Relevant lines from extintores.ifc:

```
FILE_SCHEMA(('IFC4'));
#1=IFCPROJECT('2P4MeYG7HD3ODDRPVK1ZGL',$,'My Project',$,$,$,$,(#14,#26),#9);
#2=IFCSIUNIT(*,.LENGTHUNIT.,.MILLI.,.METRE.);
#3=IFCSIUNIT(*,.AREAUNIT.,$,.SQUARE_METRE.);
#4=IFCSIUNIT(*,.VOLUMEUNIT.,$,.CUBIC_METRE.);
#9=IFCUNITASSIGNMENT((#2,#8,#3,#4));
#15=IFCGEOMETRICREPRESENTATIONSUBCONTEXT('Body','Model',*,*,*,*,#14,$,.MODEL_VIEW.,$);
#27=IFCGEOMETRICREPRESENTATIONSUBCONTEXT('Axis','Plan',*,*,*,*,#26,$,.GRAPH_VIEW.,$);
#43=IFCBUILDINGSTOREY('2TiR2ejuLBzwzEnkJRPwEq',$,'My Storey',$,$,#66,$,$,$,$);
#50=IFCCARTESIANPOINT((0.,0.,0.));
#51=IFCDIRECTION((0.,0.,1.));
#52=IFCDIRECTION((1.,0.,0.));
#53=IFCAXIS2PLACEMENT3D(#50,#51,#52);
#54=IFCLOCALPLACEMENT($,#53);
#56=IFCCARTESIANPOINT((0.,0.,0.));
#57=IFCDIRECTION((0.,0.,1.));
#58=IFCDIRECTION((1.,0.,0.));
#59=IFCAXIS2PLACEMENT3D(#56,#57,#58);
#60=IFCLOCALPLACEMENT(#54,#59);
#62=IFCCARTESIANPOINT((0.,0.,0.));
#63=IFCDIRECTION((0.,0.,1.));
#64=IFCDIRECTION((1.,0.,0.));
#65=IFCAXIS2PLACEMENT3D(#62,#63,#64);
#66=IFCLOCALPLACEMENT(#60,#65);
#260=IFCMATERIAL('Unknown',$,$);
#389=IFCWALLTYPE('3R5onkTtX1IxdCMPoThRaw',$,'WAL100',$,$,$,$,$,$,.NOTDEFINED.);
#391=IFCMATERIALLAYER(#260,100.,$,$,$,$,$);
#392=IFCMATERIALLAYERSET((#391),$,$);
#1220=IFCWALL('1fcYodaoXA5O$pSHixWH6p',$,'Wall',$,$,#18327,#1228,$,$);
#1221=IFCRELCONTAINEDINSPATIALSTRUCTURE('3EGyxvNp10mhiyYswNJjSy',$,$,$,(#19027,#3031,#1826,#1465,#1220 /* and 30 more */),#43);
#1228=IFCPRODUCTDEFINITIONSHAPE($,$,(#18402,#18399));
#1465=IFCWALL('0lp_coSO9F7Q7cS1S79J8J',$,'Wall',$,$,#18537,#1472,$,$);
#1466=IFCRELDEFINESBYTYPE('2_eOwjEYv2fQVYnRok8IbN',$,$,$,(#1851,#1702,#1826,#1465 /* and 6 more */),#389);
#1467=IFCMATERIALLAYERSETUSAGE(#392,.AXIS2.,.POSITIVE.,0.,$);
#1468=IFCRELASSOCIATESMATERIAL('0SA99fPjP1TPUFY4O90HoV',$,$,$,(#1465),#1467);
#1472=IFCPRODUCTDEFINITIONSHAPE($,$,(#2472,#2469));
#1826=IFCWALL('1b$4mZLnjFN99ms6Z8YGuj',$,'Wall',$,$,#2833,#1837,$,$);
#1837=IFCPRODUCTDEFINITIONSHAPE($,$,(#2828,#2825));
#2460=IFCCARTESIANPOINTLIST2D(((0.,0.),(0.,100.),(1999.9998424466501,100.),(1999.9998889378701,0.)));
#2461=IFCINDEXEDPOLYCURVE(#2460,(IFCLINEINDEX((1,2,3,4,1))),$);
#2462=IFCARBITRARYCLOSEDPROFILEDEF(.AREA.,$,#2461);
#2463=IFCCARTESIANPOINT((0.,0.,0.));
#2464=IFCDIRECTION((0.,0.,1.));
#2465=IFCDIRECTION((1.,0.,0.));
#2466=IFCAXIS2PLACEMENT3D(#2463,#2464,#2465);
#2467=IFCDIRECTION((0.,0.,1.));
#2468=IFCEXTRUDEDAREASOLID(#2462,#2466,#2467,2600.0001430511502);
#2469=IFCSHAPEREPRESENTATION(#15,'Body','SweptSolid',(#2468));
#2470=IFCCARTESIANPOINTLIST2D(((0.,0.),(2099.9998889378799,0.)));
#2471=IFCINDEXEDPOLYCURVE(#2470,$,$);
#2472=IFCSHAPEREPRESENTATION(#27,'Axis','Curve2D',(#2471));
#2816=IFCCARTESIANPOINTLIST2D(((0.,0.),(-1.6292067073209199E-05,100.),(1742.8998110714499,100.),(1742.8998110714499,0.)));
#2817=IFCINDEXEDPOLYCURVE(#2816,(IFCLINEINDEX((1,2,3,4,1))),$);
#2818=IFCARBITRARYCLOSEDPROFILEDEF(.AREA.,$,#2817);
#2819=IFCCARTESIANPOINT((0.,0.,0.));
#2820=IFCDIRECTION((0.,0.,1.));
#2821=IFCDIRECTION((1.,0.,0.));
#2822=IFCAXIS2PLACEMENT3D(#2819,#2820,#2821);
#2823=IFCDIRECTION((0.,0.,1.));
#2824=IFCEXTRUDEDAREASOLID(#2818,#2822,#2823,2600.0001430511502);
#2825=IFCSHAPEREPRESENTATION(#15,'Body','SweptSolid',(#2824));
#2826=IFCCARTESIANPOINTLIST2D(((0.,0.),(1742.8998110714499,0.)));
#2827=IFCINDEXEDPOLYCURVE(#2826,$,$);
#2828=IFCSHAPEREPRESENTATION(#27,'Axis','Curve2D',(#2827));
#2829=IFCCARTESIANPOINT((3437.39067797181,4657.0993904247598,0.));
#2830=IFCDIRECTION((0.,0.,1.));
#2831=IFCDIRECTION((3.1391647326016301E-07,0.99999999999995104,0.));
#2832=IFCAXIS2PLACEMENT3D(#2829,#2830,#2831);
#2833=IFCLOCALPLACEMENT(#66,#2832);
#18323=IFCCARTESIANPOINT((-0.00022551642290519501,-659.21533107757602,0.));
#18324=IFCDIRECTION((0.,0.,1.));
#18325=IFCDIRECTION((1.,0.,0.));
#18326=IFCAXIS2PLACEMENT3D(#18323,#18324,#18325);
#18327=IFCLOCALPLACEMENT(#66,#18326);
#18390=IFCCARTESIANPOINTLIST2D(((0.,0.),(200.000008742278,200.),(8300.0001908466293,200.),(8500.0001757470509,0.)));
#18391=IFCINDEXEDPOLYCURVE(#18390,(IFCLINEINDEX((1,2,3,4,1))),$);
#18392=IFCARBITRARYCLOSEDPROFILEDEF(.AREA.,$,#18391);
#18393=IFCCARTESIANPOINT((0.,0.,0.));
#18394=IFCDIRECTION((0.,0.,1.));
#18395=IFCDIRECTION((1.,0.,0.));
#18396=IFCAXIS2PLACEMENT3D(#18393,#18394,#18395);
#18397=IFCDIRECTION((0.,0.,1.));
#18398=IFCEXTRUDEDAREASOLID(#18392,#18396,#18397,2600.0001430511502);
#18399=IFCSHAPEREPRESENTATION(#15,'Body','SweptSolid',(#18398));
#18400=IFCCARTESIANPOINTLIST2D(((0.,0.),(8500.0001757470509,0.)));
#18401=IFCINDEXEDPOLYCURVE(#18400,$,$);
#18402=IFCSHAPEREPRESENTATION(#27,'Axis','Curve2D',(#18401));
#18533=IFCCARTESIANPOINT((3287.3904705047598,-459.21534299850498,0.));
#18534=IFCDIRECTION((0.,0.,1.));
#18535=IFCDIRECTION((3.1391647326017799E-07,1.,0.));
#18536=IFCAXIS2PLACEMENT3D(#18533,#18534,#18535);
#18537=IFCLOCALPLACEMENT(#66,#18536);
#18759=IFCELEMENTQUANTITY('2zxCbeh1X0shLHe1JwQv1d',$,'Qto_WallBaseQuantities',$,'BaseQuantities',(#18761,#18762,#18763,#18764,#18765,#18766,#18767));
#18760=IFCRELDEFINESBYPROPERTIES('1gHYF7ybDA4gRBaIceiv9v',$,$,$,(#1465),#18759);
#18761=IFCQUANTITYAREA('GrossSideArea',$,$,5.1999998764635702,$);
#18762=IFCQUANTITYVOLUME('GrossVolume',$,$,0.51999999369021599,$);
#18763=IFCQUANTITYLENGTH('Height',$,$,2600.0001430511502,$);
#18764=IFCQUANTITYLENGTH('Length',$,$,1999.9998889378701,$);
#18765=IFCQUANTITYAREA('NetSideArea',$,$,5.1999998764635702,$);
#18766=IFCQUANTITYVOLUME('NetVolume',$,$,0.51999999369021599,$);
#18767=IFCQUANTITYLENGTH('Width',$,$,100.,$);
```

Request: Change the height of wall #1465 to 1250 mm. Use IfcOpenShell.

```python
import ifcopenshell
import ifcopenshell.api.pset
import ifcopenshell.geom
import ifcopenshell.util.element
import ifcopenshell.util.representation
import ifcopenshell.util.shape
import ifcopenshell.util.unit

model = ifcopenshell.open("extintores.ifc")
unit_scale = ifcopenshell.util.unit.calculate_unit_scale(model)
area_scale = ifcopenshell.util.unit.calculate_unit_scale(model, "AREAUNIT")
volume_scale = ifcopenshell.util.unit.calculate_unit_scale(model, "VOLUMEUNIT")
settings = ifcopenshell.geom.settings()


def volume(element):
    """Net volume in cubic metres, openings subtracted."""
    shape = ifcopenshell.geom.create_shape(settings, element)
    return ifcopenshell.util.shape.get_volume(shape.geometry)


wall = model.by_guid("0lp_coSO9F7Q7cS1S79J8J")
before = volume(wall)

body = ifcopenshell.util.representation.get_representation(wall, "Model", "Body")
solid = body.Items[0]
old_height = solid.Depth
solid.Depth = 1250.0
after = volume(wall)
thickness = 0.1  # wall thickness in metres

# Update the stored height, areas and volumes.
qto = model.by_id(ifcopenshell.util.element.get_pset(wall, "Qto_WallBaseQuantities", should_inherit=False)["id"])
ifcopenshell.api.pset.edit_qto(model, qto=qto, properties={
    "GrossSideArea": ifcopenshell.util.element.get_pset(wall, "Qto_WallBaseQuantities", "GrossSideArea") * solid.Depth / old_height,
    "GrossVolume": ifcopenshell.util.element.get_pset(wall, "Qto_WallBaseQuantities", "GrossVolume") * solid.Depth / old_height,
    "Height": solid.Depth,
    "NetSideArea": after / thickness / area_scale,
    "NetVolume": after / volume_scale,
})

print(f"height {old_height:g} -> {solid.Depth:g}, volume {before:.3f} -> {after:.3f} m3")

model.write("extintores_edited.ifc")
```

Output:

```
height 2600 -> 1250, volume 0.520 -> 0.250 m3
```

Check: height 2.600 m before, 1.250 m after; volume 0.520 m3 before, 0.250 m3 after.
